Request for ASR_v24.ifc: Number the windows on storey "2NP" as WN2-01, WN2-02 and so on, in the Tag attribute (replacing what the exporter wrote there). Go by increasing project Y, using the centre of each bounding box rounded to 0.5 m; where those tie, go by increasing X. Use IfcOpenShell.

First a look at what the model holds.

```python
import ifcopenshell
import ifcopenshell.util.element
import ifcopenshell.util.placement

model = ifcopenshell.open("ASR_v24.ifc")
print(model.schema)
storey = next(s for s in model.by_type("IfcBuildingStorey") if s.Name == "2NP")
windows = [e for e in ifcopenshell.util.element.get_decomposition(storey) if e.is_a("IfcWindow")]
for e in sorted(windows, key=lambda e: e.id()):
    origin = ifcopenshell.util.placement.get_local_placement(e.ObjectPlacement)[:3, 3]
    print(e.id(), e.Tag, e.Name, origin.round(2) + 0.0, sep=" | ")
```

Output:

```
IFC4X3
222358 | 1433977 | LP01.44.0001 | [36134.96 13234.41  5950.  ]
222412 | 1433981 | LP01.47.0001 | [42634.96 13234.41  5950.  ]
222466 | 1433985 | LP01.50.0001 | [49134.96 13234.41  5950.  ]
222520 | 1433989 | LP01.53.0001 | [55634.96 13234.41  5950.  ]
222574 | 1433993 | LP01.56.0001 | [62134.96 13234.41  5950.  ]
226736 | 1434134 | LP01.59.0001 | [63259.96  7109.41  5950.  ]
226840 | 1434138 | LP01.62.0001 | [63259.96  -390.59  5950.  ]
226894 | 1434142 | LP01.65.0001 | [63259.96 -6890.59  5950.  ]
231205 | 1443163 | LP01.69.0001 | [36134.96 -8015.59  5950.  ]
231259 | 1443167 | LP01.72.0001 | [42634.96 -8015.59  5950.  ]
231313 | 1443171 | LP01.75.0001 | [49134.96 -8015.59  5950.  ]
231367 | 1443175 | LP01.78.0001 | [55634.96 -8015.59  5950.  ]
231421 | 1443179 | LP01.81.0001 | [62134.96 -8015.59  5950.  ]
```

```python
import ifcopenshell
import ifcopenshell.geom
import ifcopenshell.util.element
import ifcopenshell.util.shape

model = ifcopenshell.open("ASR_v24.ifc")
settings = ifcopenshell.geom.settings()
settings.set("use-world-coords", True)


def centre(element):
    shape = ifcopenshell.geom.create_shape(settings, element)
    return ifcopenshell.util.shape.get_bbox_centroid(shape.geometry)


storey = next(s for s in model.by_type("IfcBuildingStorey") if s.Name == "2NP")
windows = [e for e in ifcopenshell.util.element.get_decomposition(storey) if e.is_a("IfcWindow")]

# Insertion points can sit at a corner or the storey origin, so sort by the geometry (in metres).
centres = {e: centre(e) for e in windows}
windows.sort(key=lambda e: (round(centres[e][1] / 0.5), centres[e][0]))

for i, e in enumerate(windows, start=1):
    number = f"WN2-{i:02d}"
    e.Tag = number
    print(e.id(), number)

model.write("ASR_v24_edited.ifc")
```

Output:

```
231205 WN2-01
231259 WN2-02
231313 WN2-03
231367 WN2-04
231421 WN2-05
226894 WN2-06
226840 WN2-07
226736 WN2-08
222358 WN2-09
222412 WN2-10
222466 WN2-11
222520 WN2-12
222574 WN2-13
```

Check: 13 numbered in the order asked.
